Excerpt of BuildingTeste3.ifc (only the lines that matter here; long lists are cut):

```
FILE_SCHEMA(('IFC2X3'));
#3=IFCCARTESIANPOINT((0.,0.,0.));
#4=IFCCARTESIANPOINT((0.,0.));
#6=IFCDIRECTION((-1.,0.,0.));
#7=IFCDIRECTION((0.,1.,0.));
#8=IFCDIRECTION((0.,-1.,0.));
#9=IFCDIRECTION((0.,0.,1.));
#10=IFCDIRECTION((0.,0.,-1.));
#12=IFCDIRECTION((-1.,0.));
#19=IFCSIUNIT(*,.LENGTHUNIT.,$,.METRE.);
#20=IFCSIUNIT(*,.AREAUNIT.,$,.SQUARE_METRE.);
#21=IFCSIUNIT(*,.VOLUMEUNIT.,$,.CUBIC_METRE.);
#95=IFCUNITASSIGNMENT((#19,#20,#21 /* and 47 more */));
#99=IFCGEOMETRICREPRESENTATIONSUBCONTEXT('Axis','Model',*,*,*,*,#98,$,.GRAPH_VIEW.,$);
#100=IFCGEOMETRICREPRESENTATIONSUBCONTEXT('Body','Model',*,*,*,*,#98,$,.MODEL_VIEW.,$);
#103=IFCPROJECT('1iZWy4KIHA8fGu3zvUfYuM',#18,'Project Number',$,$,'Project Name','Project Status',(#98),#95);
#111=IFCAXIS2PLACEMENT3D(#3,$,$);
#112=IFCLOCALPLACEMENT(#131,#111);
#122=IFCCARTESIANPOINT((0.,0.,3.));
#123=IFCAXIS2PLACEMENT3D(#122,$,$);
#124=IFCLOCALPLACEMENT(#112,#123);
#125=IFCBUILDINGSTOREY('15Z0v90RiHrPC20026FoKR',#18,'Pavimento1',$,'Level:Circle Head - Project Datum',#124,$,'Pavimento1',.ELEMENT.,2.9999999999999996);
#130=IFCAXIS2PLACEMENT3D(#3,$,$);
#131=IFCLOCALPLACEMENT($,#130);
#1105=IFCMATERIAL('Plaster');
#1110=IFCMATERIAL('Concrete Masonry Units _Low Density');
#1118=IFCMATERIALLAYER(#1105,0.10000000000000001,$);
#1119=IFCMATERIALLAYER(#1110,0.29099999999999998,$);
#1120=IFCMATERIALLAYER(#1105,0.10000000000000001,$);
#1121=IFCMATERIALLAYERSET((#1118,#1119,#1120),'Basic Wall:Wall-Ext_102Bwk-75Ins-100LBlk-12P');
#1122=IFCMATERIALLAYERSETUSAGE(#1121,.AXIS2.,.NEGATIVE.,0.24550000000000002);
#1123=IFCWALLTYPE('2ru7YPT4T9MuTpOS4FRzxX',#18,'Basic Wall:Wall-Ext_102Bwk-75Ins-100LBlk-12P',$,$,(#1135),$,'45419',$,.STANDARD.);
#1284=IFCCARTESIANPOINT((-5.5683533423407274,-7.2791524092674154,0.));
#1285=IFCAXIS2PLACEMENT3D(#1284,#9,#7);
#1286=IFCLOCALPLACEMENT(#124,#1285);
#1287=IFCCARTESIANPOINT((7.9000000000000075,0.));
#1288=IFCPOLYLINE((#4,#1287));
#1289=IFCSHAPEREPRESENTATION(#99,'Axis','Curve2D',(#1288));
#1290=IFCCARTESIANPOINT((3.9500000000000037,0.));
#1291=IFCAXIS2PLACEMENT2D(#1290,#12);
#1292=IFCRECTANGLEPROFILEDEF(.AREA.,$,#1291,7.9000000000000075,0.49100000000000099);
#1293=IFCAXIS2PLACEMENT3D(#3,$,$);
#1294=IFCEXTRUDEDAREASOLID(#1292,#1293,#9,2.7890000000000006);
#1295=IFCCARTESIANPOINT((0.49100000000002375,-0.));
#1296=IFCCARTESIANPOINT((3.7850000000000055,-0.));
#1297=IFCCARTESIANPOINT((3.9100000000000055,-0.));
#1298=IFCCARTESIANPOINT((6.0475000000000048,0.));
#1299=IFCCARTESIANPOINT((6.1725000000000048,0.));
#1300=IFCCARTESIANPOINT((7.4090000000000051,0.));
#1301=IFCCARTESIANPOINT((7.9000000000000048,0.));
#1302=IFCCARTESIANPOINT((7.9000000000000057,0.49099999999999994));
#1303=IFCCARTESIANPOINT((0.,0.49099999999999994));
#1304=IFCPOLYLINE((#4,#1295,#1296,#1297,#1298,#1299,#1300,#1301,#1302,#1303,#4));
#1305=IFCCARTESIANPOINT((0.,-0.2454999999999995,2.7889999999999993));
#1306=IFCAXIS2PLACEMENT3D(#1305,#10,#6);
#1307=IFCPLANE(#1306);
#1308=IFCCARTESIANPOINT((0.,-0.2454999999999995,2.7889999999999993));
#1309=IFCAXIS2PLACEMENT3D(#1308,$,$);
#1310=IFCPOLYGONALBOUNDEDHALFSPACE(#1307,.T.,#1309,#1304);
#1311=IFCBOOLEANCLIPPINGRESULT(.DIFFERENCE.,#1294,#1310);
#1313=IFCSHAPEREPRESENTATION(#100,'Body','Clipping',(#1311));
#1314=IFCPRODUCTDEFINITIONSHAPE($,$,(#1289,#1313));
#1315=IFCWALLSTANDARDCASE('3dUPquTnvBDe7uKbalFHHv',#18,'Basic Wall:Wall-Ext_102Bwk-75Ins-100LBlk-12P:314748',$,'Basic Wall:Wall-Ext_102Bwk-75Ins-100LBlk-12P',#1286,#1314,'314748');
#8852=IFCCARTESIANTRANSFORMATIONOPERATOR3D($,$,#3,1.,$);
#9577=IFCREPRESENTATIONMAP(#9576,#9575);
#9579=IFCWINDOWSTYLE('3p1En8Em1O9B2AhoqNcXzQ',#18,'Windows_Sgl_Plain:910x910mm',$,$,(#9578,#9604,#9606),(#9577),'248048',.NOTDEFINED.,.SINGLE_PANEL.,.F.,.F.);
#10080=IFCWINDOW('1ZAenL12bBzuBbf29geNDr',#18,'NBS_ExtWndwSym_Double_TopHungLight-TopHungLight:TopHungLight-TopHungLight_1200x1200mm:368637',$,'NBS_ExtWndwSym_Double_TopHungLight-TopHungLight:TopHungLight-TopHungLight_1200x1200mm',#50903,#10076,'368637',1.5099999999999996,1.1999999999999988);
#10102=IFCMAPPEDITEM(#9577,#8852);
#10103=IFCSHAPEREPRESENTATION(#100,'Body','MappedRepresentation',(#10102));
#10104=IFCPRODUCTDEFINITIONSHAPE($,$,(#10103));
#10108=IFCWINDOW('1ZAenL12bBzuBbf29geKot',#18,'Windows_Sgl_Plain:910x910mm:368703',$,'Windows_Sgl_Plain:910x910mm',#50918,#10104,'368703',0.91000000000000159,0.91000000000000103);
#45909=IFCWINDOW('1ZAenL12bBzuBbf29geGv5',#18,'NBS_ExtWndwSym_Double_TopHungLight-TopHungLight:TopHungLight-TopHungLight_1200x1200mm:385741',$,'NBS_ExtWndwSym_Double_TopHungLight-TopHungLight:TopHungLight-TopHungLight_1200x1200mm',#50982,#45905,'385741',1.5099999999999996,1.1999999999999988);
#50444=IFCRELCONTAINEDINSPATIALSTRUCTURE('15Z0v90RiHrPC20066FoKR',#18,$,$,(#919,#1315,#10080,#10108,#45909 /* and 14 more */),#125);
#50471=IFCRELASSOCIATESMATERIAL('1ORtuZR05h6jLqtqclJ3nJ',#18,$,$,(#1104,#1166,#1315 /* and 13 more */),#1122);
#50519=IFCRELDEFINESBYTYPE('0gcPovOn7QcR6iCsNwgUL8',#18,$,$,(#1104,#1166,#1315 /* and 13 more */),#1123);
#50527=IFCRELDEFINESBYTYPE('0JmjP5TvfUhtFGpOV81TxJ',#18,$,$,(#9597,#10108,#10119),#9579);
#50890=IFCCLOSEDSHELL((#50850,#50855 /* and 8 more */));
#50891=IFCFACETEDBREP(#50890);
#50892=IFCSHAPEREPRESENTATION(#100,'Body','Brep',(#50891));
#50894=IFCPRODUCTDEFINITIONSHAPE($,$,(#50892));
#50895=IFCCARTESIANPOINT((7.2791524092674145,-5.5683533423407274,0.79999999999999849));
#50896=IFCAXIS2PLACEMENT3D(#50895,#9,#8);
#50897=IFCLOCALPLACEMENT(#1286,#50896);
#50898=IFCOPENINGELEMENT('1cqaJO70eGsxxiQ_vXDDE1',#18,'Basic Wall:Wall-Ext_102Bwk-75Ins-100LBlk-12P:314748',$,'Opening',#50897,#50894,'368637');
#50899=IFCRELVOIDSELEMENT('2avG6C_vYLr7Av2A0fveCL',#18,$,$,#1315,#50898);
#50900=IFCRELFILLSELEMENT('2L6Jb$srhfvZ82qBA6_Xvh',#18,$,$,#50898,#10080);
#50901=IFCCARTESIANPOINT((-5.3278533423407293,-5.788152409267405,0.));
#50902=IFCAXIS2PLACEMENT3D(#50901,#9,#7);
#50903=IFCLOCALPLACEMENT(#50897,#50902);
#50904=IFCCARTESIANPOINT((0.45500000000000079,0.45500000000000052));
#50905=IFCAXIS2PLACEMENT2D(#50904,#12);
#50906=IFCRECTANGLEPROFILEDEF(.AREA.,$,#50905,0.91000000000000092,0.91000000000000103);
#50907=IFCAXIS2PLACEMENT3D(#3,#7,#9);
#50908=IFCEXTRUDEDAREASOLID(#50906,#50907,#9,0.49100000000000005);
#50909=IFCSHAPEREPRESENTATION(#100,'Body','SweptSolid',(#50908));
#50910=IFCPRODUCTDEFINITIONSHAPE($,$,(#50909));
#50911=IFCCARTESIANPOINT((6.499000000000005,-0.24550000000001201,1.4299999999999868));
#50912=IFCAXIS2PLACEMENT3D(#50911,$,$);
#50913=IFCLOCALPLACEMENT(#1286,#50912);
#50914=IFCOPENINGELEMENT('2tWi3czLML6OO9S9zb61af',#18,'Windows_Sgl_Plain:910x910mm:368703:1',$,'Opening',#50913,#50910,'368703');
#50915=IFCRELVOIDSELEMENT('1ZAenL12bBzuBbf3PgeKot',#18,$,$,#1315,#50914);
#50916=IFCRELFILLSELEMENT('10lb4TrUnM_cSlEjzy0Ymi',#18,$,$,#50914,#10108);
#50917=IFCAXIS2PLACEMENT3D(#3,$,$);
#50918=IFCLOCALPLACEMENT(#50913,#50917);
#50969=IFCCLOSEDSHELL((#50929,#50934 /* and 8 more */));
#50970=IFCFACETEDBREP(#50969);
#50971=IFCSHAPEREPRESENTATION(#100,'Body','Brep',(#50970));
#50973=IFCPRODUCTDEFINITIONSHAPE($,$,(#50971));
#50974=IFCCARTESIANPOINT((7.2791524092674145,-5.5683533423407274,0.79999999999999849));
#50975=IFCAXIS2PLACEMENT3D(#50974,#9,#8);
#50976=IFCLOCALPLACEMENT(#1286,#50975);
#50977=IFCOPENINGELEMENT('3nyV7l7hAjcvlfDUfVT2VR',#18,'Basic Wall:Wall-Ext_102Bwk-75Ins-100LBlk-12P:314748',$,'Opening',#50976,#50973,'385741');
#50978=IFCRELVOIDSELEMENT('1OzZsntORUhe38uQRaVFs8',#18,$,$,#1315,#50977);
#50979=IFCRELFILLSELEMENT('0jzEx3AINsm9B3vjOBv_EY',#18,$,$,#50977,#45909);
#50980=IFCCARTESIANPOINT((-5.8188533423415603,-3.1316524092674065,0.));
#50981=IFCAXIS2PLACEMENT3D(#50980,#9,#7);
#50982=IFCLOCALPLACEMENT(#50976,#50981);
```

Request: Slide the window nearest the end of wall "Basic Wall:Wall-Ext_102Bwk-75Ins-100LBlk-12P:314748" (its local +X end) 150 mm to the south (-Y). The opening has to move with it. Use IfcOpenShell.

```python
import ifcopenshell
import ifcopenshell.api.geometry
import ifcopenshell.util.placement
import ifcopenshell.util.unit

model = ifcopenshell.open("BuildingTeste3.ifc")
unit_scale = ifcopenshell.util.unit.calculate_unit_scale(model)

window = model.by_guid("1ZAenL12bBzuBbf29geKot")
opening = window.FillsVoids[0].RelatingOpeningElement
wall = opening.VoidsElements[0].RelatingBuildingElement

wall_matrix = ifcopenshell.util.placement.get_local_placement(wall.ObjectPlacement)
shift = wall_matrix[:3, 0] * -0.15 / unit_scale
before = ifcopenshell.util.placement.get_local_placement(window.ObjectPlacement)[:3, 3].copy()

# The window is placed relative to its opening, so it follows when the opening moves.
matrix = ifcopenshell.util.placement.get_local_placement(opening.ObjectPlacement)
matrix[:3, 3] += shift
ifcopenshell.api.geometry.edit_object_placement(
    model, product=opening, matrix=matrix, is_si=False, should_transform_children=True
)

after = ifcopenshell.util.placement.get_local_placement(window.ObjectPlacement)[:3, 3]
print("window moved by", (after - before).round(3) + 0.0)

model.write("BuildingTeste3_updated.ifc")
```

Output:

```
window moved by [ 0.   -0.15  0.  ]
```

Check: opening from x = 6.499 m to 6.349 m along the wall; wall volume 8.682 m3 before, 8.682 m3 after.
